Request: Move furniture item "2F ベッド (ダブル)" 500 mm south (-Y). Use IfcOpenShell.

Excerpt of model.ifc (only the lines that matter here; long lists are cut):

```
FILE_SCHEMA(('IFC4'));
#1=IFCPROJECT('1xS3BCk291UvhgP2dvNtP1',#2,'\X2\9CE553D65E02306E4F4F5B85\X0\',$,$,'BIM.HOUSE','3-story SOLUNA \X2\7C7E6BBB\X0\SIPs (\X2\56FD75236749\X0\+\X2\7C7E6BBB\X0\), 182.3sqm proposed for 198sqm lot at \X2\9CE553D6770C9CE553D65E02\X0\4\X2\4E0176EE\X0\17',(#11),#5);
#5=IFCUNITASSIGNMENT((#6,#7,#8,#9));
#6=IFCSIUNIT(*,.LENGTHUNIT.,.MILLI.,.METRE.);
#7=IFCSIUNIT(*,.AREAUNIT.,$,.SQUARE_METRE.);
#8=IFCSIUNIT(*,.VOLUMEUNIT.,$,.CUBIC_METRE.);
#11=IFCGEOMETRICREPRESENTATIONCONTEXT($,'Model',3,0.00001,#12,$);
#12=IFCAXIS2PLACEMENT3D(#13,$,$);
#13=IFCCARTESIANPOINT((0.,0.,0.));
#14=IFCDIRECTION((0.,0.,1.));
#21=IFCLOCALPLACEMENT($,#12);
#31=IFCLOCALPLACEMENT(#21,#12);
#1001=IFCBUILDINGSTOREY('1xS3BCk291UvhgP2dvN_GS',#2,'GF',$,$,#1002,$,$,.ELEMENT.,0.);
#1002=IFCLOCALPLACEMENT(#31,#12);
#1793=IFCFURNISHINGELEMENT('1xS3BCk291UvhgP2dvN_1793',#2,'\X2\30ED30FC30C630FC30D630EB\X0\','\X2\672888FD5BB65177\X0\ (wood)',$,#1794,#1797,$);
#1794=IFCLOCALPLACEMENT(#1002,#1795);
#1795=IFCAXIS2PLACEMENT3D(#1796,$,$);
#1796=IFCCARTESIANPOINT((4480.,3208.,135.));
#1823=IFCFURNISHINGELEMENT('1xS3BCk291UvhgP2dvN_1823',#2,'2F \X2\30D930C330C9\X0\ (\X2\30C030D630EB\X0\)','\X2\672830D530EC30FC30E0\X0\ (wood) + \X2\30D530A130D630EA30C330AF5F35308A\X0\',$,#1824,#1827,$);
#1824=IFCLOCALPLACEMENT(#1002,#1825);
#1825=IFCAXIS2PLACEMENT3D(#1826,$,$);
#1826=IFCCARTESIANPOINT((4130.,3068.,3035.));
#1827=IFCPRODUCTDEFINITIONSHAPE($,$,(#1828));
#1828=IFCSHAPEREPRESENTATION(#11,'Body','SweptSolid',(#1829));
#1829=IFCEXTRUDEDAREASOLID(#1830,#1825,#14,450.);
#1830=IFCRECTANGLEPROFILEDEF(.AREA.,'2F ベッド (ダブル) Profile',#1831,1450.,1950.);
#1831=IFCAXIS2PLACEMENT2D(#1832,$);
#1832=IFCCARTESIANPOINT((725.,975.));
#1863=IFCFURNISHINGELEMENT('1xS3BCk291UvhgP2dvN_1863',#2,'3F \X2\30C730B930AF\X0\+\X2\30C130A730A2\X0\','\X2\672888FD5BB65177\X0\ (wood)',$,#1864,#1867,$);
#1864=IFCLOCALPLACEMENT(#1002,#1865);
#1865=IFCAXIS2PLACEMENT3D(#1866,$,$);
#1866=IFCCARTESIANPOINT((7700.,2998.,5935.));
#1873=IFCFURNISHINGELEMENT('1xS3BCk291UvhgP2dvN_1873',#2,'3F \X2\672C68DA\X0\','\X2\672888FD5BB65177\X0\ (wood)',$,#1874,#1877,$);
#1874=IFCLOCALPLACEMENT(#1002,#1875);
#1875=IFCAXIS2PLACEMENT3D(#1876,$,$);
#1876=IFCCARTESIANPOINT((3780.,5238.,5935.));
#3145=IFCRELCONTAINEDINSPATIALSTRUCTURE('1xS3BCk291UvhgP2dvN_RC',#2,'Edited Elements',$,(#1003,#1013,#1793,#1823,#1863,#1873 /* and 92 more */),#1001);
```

```python
import ifcopenshell
import ifcopenshell.api.geometry
import ifcopenshell.util.placement

model = ifcopenshell.open("model.ifc")

item = model.by_guid("1xS3BCk291UvhgP2dvN_1823")
matrix = ifcopenshell.util.placement.get_local_placement(item.ObjectPlacement)
matrix[1, 3] -= 500.0
ifcopenshell.api.geometry.edit_object_placement(model, product=item, matrix=matrix, is_si=False)

print(ifcopenshell.util.placement.get_local_placement(item.ObjectPlacement).round(3) + 0.0)

model.write("model-out.ifc")
```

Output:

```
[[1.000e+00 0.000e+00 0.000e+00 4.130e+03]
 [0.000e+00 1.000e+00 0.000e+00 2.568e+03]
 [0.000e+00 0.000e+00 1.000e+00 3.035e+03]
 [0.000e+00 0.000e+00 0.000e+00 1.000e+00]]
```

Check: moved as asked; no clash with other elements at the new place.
